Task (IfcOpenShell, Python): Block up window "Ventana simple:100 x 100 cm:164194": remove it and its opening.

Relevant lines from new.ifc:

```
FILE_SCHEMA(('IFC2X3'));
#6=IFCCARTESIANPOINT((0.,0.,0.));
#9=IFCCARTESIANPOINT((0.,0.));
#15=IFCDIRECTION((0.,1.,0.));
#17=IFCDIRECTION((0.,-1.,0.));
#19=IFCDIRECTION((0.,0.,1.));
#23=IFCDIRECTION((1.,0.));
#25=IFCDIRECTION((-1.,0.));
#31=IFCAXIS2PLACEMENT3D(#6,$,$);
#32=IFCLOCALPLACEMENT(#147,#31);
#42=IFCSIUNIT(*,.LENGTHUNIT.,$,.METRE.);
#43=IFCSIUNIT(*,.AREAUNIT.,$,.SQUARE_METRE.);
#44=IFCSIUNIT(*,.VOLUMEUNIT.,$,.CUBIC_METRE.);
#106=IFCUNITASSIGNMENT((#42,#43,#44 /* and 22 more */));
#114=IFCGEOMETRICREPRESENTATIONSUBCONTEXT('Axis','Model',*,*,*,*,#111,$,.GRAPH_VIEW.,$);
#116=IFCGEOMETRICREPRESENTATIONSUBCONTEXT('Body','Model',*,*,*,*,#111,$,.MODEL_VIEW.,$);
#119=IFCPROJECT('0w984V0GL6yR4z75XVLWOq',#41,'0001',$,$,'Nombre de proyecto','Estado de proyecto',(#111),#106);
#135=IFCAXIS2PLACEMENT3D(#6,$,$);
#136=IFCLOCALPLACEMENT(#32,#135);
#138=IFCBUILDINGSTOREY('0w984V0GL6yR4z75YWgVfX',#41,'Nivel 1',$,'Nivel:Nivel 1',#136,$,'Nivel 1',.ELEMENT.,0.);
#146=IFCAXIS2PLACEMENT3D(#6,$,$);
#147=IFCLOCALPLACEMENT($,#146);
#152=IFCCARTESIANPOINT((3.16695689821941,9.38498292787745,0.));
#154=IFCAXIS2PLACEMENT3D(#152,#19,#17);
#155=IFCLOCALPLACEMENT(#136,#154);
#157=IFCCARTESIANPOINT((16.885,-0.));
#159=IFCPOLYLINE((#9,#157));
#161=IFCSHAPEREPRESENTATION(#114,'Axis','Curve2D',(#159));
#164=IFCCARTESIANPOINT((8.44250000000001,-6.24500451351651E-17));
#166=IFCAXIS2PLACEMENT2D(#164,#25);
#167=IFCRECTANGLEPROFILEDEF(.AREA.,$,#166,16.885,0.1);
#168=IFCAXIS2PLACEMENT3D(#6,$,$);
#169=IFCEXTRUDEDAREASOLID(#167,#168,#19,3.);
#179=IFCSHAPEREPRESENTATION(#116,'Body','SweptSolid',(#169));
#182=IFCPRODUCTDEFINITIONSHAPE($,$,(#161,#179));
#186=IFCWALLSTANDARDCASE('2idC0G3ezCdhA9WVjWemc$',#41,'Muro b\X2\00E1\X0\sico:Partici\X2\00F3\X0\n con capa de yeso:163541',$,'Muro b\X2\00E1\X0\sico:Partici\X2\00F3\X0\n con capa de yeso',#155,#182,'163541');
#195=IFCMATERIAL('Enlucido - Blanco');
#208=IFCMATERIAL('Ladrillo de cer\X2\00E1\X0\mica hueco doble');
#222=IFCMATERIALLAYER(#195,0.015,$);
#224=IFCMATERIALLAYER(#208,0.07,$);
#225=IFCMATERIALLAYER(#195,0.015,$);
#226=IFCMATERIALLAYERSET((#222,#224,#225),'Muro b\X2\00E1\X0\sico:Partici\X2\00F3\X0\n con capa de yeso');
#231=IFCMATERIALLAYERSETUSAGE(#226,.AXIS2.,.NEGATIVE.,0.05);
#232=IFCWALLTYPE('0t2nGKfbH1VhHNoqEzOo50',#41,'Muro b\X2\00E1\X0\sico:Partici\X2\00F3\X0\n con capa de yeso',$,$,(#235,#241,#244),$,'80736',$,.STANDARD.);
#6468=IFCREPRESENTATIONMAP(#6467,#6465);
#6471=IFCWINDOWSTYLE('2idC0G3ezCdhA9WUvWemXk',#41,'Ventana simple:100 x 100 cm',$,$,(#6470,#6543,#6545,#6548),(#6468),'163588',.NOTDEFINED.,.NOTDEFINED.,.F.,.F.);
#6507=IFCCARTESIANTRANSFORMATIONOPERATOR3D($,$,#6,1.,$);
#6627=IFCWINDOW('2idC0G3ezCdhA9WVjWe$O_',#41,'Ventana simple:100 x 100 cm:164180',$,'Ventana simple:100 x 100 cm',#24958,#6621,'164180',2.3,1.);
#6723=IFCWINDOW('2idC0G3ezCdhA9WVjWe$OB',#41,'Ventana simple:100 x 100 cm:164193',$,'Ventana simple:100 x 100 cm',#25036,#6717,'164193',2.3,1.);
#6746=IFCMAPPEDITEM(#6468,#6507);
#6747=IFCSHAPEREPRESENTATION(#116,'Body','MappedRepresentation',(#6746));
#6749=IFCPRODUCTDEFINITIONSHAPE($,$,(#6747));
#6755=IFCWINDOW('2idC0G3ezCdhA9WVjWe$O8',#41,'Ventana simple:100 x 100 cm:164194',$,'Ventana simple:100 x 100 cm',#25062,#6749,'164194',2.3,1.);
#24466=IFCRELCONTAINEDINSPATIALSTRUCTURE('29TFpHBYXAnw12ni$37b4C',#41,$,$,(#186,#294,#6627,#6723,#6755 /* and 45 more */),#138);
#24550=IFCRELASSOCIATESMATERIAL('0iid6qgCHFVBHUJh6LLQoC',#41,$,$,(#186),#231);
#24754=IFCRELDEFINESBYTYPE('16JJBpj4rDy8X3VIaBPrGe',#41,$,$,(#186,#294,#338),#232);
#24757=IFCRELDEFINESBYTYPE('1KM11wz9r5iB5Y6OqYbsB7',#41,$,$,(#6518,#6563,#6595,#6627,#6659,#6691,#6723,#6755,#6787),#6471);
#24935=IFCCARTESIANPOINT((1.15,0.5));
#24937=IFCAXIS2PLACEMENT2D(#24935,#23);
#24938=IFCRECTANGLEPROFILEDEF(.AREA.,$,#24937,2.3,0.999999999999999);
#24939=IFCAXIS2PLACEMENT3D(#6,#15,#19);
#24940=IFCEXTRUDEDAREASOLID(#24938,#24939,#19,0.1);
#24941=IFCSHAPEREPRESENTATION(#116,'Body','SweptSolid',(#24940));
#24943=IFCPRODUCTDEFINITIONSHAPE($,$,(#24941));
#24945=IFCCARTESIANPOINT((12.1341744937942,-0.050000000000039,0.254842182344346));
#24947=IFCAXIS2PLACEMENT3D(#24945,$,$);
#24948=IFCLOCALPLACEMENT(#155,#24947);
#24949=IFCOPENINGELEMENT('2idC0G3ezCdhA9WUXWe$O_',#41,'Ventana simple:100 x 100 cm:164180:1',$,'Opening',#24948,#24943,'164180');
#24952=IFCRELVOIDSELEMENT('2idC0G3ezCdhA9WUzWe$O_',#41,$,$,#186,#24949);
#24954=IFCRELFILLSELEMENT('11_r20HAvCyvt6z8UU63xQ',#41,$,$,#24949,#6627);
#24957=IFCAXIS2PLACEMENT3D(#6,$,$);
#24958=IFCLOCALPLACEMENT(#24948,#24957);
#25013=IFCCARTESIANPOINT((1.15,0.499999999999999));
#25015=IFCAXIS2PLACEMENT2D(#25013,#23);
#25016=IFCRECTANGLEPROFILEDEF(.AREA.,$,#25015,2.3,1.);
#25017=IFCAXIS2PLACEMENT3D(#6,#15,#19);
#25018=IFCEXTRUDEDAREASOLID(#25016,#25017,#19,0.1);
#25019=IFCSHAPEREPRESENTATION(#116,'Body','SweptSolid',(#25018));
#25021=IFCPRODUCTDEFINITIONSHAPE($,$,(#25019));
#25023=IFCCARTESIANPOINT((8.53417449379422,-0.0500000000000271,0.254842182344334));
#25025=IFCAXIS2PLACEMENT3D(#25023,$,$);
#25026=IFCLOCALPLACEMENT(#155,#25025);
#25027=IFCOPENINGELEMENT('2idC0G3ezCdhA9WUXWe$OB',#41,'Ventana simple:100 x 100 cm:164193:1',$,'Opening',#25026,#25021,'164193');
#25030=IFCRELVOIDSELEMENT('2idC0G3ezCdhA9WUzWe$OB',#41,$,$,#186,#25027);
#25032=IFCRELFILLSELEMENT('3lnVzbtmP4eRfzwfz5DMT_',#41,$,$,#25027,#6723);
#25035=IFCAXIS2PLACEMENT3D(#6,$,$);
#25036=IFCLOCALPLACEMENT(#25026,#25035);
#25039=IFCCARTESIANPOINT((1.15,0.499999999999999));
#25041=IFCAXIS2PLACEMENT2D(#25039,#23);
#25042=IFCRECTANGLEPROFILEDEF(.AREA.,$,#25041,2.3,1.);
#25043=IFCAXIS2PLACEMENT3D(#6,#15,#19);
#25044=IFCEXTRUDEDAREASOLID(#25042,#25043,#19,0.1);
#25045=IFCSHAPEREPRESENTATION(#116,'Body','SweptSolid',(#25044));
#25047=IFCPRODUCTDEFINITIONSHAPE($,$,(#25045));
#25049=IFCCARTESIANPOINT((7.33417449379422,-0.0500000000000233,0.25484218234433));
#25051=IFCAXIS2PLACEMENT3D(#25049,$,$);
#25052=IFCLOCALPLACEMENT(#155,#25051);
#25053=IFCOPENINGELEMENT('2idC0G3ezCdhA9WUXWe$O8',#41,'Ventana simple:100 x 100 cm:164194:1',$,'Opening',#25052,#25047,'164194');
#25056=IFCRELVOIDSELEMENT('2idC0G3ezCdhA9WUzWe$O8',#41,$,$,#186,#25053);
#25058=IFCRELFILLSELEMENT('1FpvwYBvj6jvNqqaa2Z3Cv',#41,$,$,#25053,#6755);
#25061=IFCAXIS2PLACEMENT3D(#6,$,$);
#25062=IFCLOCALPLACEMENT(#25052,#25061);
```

```python
import ifcopenshell
import ifcopenshell.api.feature
import ifcopenshell.api.root
import ifcopenshell.geom
import ifcopenshell.util.shape

model = ifcopenshell.open("new.ifc")
settings = ifcopenshell.geom.settings()


def volume(element):
    """Net volume in cubic metres, openings subtracted."""
    shape = ifcopenshell.geom.create_shape(settings, element)
    return ifcopenshell.util.shape.get_volume(shape.geometry)


window = model.by_guid("2idC0G3ezCdhA9WVjWe$O8")
opening = window.FillsVoids[0].RelatingOpeningElement
wall = opening.VoidsElements[0].RelatingBuildingElement
before = volume(wall)

ifcopenshell.api.root.remove_product(model, product=window)
ifcopenshell.api.feature.remove_feature(model, feature=opening)

after = volume(wall)

print(f"wall volume {before:.3f} -> {after:.3f} m3")

model.write("new_v2.ifc")
```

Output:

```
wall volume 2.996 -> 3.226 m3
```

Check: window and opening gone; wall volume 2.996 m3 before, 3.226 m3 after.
